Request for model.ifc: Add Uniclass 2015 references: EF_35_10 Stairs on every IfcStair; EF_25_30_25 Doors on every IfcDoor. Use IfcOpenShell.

First a look at what the model holds.

```python
import ifcopenshell

model = ifcopenshell.open("model.ifc")
print(model.schema)
print("classifications:", [c.Name for c in model.by_type("IfcClassification")])
for ifc_class in ("IfcDoor", "IfcRoof", "IfcStair", "IfcWall", "IfcWindow"):
    print(ifc_class, len(model.by_type(ifc_class)))
```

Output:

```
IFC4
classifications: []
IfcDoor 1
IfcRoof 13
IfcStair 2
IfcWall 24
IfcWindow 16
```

```python
import ifcopenshell
import ifcopenshell.api.classification

model = ifcopenshell.open("model.ifc")

system = ifcopenshell.api.classification.add_classification(model, classification="Uniclass 2015")

codes = {
    "IfcStair": ("EF_35_10", "Stairs"),
    "IfcDoor": ("EF_25_30_25", "Doors"),
}
for ifc_class, (code, name) in codes.items():
    products = model.by_type(ifc_class)
    ifcopenshell.api.classification.add_reference(
        model, products=products, classification=system, identification=code, name=name
    )
    print(code, len(products))

model.write("model_edited.ifc")
```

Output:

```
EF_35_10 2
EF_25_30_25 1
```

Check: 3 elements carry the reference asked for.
